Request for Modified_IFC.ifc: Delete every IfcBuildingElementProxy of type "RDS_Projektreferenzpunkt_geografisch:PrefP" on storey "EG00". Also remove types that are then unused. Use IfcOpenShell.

First a look at what the model holds.

```python
import ifcopenshell
import ifcopenshell.util.element

model = ifcopenshell.open("Modified_IFC.ifc")
print(model.schema)
storey = next(s for s in model.by_type("IfcBuildingStorey") if s.Name == "EG00")
proxies = [e for e in ifcopenshell.util.element.get_decomposition(storey) if e.is_a("IfcBuildingElementProxy")]
seen = {}
for e in proxies:
    element_type = ifcopenshell.util.element.get_type(e)
    name = element_type.Name if element_type not in (None, e) else None
    seen[name] = seen.get(name, 0) + 1
for name, count in sorted(seen.items(), key=str):
    print(count, "x", name)
```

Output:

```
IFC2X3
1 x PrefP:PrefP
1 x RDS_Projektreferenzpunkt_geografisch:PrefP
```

```python
import ifcopenshell
import ifcopenshell.api.root
import ifcopenshell.util.element

model = ifcopenshell.open("Modified_IFC.ifc")

storey = next(s for s in model.by_type("IfcBuildingStorey") if s.Name == "EG00")
proxies = [e for e in ifcopenshell.util.element.get_decomposition(storey) if e.is_a("IfcBuildingElementProxy")]
targets = [e for e in proxies if (t := ifcopenshell.util.element.get_type(e)) not in (None, e) and t.Name == "RDS_Projektreferenzpunkt_geografisch:PrefP"]
types = {ifcopenshell.util.element.get_type(e) for e in targets} - {None, *targets}

for e in targets:
    ifcopenshell.api.root.remove_product(model, product=e)
print(len(targets), "removed")

unused = [t for t in types if not ifcopenshell.util.element.get_types(t)]
for t in unused:
    ifcopenshell.api.root.remove_product(model, product=t)
print(len(unused), "unused types removed")

model.write("Modified_IFC_v2.ifc")
```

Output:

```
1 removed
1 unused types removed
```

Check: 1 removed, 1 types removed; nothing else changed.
